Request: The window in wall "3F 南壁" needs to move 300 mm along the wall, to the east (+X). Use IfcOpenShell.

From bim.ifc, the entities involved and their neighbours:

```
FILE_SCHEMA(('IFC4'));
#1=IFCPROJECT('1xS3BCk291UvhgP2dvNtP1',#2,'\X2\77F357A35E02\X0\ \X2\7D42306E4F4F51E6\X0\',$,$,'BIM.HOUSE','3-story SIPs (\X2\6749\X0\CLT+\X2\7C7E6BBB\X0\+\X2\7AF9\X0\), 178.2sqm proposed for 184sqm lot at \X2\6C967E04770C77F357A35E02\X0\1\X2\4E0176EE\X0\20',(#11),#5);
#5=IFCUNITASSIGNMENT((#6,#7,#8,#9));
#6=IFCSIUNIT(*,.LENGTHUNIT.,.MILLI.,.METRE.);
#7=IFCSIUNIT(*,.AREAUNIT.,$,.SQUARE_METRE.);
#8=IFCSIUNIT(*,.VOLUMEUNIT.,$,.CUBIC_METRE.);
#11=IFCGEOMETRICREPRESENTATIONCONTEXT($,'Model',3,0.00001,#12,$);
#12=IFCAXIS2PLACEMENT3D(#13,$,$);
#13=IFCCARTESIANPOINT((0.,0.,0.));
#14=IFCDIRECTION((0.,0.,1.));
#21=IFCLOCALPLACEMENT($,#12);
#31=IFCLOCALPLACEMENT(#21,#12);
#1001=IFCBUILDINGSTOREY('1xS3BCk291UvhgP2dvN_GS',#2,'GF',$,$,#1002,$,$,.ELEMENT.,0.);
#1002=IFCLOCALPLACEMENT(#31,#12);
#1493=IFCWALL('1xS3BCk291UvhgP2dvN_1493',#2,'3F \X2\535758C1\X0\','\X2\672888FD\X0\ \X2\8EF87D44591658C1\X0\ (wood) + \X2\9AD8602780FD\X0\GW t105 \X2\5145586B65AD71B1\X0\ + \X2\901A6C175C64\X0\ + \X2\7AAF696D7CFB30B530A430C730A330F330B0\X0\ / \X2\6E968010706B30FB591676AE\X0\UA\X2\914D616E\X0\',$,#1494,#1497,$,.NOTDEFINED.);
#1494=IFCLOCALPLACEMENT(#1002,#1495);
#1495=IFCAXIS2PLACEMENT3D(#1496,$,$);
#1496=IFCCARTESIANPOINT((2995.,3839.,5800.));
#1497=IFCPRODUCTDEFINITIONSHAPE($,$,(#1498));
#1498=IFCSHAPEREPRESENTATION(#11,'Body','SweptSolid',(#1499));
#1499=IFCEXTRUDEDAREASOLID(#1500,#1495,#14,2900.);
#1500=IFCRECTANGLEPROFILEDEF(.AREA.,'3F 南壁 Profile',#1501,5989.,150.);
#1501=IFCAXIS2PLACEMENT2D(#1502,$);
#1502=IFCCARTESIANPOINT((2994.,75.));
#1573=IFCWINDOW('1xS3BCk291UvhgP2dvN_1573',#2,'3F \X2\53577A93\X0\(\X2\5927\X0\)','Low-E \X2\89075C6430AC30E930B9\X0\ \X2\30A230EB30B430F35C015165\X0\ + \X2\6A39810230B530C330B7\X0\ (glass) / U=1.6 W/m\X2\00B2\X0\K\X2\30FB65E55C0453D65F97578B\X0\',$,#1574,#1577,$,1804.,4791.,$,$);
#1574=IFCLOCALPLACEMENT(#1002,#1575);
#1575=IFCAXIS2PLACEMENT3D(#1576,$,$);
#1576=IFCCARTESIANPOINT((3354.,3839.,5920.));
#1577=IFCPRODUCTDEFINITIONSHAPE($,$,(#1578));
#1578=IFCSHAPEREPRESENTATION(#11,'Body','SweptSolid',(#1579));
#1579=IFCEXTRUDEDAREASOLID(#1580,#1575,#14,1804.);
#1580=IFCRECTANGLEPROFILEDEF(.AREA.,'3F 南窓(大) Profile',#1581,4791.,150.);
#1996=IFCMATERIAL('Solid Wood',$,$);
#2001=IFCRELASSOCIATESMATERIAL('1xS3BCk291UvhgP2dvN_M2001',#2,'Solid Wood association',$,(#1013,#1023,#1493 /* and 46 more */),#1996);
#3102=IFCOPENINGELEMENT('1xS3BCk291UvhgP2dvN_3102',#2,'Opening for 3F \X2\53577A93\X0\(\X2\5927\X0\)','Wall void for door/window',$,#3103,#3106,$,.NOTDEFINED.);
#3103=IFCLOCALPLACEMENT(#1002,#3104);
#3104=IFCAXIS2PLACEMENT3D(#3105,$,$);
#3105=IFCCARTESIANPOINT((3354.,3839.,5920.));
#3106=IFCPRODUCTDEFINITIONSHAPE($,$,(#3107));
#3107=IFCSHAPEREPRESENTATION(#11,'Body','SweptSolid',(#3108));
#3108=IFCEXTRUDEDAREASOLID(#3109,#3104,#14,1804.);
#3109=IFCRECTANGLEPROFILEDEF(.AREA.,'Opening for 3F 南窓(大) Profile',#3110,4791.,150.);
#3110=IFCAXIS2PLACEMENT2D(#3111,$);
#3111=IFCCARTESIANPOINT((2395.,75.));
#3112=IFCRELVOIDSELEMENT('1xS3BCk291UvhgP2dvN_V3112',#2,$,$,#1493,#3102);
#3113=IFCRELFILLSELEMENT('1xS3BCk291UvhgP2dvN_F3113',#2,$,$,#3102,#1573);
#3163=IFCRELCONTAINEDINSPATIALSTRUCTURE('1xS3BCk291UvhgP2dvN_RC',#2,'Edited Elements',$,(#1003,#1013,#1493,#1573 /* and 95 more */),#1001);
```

```python
import ifcopenshell
import ifcopenshell.api.geometry
import ifcopenshell.util.placement
import ifcopenshell.util.unit

model = ifcopenshell.open("bim.ifc")
unit_scale = ifcopenshell.util.unit.calculate_unit_scale(model)

window = model.by_guid("1xS3BCk291UvhgP2dvN_1573")
opening = window.FillsVoids[0].RelatingOpeningElement
wall = opening.VoidsElements[0].RelatingBuildingElement

wall_matrix = ifcopenshell.util.placement.get_local_placement(wall.ObjectPlacement)
shift = wall_matrix[:3, 0] * 0.3 / unit_scale
before = ifcopenshell.util.placement.get_local_placement(window.ObjectPlacement)[:3, 3].copy()

# The window is not placed relative to its opening, so move both.
for product in (opening, window):
    matrix = ifcopenshell.util.placement.get_local_placement(product.ObjectPlacement)
    matrix[:3, 3] += shift
    ifcopenshell.api.geometry.edit_object_placement(model, product=product, matrix=matrix, is_si=False)

after = ifcopenshell.util.placement.get_local_placement(window.ObjectPlacement)[:3, 3]
print("window moved by", (after - before).round(3) + 0.0)

model.write("bim_updated.ifc")
```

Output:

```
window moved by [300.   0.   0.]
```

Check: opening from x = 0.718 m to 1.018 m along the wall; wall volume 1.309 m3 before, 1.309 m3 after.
